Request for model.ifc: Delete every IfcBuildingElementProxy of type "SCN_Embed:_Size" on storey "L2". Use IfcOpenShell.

First a look at what the model holds.

```python
import ifcopenshell
import ifcopenshell.util.element

model = ifcopenshell.open("model.ifc")
print(model.schema)
storey = next(s for s in model.by_type("IfcBuildingStorey") if s.Name == "L2")
proxies = [e for e in ifcopenshell.util.element.get_decomposition(storey) if e.is_a("IfcBuildingElementProxy")]
seen = {}
for e in proxies:
    element_type = ifcopenshell.util.element.get_type(e)
    name = element_type.Name if element_type not in (None, e) else None
    seen[name] = seen.get(name, 0) + 1
for name, count in sorted(seen.items(), key=str):
    print(count, "x", name)
```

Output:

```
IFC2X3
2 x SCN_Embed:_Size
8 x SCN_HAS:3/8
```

```python
import ifcopenshell
import ifcopenshell.api.root
import ifcopenshell.util.element

model = ifcopenshell.open("model.ifc")

storey = next(s for s in model.by_type("IfcBuildingStorey") if s.Name == "L2")
proxies = [e for e in ifcopenshell.util.element.get_decomposition(storey) if e.is_a("IfcBuildingElementProxy")]
targets = [e for e in proxies if (t := ifcopenshell.util.element.get_type(e)) not in (None, e) and t.Name == "SCN_Embed:_Size"]

for e in targets:
    ifcopenshell.api.root.remove_product(model, product=e)
print(len(targets), "removed")

model.write("model-out.ifc")
```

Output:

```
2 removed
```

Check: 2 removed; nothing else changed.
